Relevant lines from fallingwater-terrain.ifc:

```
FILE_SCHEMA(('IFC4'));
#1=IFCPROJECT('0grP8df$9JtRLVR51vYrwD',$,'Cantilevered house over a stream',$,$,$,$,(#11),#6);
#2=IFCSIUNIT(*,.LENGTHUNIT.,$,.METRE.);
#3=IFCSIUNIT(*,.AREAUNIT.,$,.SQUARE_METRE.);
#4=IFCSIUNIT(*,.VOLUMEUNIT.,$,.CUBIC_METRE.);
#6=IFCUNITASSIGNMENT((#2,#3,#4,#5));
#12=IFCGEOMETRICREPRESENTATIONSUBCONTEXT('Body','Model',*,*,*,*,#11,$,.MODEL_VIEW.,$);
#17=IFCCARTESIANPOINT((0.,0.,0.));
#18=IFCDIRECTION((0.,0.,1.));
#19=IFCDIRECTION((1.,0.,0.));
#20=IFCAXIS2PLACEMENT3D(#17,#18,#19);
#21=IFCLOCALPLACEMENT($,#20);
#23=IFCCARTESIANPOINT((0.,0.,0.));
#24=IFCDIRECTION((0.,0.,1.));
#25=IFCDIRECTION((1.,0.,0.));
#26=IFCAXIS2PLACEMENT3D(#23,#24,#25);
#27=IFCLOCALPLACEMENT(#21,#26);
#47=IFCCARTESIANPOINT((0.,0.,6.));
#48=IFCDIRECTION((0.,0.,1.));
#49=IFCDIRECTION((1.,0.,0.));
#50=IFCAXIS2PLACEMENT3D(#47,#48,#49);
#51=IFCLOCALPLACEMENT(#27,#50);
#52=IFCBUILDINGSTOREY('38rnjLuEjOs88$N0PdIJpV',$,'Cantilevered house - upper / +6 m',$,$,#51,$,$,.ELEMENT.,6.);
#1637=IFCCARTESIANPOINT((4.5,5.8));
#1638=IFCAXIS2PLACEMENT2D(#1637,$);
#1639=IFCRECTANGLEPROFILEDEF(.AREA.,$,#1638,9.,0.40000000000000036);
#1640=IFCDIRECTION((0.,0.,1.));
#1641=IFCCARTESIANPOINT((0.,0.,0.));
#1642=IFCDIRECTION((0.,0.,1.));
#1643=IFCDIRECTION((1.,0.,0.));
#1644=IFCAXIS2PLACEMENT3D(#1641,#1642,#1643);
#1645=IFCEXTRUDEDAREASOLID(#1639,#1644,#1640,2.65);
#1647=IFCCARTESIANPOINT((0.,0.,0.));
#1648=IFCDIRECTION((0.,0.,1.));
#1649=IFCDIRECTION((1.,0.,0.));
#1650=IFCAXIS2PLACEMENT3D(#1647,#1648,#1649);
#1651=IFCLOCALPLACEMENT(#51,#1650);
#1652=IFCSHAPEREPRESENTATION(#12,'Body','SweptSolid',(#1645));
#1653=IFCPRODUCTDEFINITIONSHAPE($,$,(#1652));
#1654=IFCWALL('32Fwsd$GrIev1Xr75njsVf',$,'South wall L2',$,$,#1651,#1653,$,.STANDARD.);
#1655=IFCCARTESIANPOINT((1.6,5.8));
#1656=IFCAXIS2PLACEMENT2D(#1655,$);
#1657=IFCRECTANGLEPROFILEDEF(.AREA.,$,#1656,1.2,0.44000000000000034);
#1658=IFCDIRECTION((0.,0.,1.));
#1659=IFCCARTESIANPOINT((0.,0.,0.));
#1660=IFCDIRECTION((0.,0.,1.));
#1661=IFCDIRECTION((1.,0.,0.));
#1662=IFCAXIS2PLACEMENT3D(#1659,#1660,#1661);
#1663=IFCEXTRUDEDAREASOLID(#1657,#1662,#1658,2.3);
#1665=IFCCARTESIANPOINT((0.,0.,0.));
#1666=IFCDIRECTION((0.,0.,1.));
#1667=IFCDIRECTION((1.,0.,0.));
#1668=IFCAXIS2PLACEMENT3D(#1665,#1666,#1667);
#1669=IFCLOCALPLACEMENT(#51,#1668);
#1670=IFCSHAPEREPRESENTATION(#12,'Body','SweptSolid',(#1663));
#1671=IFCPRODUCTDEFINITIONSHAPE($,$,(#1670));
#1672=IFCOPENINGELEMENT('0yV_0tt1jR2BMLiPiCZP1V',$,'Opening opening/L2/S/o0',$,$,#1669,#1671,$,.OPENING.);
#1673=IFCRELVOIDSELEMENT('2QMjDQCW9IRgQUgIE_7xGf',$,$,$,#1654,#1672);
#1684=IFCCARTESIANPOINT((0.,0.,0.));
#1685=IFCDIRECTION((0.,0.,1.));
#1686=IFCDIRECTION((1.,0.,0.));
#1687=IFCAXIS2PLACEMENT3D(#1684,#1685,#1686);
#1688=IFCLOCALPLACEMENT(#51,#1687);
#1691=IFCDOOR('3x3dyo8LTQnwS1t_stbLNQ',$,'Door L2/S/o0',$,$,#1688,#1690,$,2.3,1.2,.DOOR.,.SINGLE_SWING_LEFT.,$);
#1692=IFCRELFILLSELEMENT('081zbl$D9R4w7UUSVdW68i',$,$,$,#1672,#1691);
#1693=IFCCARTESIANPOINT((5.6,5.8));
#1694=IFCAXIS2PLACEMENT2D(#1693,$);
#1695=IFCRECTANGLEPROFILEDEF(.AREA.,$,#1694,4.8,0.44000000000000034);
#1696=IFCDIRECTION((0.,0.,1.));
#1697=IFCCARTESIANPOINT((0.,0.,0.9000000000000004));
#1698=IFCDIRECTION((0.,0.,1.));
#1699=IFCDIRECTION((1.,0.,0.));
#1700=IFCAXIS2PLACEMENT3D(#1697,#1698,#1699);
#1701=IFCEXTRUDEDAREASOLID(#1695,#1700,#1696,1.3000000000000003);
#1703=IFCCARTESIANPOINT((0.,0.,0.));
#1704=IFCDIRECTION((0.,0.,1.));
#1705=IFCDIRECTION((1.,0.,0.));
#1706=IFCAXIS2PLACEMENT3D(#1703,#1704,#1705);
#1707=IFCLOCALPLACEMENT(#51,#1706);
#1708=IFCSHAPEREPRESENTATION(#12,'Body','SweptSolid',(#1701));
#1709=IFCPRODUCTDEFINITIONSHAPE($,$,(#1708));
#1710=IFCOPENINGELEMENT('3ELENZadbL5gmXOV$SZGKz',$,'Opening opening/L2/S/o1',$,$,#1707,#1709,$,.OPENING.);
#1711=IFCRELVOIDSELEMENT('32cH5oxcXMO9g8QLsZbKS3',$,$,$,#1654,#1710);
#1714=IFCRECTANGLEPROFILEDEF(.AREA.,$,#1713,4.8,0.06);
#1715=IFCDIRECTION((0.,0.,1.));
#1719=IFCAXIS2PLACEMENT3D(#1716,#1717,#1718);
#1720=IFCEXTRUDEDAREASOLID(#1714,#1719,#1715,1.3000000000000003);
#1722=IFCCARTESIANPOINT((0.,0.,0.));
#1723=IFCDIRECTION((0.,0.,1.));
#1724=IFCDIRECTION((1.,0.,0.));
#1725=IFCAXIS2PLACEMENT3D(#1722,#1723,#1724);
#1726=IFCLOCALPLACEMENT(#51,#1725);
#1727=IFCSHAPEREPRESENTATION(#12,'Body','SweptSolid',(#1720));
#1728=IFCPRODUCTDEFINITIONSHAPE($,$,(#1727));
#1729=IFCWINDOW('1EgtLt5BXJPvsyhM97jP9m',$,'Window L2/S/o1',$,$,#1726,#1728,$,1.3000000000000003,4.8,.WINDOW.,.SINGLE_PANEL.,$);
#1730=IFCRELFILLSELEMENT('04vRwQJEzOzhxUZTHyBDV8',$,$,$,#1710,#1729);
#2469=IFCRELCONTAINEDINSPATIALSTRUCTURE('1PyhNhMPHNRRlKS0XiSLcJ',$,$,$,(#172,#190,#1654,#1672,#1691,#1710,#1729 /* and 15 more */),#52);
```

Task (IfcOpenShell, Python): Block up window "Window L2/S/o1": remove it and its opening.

```python
import ifcopenshell
import ifcopenshell.api.feature
import ifcopenshell.api.root
import ifcopenshell.geom
import ifcopenshell.util.shape

model = ifcopenshell.open("fallingwater-terrain.ifc")
settings = ifcopenshell.geom.settings()


def volume(element):
    """Net volume in cubic metres, openings subtracted."""
    shape = ifcopenshell.geom.create_shape(settings, element)
    return ifcopenshell.util.shape.get_volume(shape.geometry)


window = model.by_guid("1EgtLt5BXJPvsyhM97jP9m")
opening = window.FillsVoids[0].RelatingOpeningElement
wall = opening.VoidsElements[0].RelatingBuildingElement
before = volume(wall)

ifcopenshell.api.root.remove_product(model, product=window)
ifcopenshell.api.feature.remove_feature(model, feature=opening)

after = volume(wall)

print(f"wall volume {before:.3f} -> {after:.3f} m3")

model.write("fallingwater-terrain_rev.ifc")
```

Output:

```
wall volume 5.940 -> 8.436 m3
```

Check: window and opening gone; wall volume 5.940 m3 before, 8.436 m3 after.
